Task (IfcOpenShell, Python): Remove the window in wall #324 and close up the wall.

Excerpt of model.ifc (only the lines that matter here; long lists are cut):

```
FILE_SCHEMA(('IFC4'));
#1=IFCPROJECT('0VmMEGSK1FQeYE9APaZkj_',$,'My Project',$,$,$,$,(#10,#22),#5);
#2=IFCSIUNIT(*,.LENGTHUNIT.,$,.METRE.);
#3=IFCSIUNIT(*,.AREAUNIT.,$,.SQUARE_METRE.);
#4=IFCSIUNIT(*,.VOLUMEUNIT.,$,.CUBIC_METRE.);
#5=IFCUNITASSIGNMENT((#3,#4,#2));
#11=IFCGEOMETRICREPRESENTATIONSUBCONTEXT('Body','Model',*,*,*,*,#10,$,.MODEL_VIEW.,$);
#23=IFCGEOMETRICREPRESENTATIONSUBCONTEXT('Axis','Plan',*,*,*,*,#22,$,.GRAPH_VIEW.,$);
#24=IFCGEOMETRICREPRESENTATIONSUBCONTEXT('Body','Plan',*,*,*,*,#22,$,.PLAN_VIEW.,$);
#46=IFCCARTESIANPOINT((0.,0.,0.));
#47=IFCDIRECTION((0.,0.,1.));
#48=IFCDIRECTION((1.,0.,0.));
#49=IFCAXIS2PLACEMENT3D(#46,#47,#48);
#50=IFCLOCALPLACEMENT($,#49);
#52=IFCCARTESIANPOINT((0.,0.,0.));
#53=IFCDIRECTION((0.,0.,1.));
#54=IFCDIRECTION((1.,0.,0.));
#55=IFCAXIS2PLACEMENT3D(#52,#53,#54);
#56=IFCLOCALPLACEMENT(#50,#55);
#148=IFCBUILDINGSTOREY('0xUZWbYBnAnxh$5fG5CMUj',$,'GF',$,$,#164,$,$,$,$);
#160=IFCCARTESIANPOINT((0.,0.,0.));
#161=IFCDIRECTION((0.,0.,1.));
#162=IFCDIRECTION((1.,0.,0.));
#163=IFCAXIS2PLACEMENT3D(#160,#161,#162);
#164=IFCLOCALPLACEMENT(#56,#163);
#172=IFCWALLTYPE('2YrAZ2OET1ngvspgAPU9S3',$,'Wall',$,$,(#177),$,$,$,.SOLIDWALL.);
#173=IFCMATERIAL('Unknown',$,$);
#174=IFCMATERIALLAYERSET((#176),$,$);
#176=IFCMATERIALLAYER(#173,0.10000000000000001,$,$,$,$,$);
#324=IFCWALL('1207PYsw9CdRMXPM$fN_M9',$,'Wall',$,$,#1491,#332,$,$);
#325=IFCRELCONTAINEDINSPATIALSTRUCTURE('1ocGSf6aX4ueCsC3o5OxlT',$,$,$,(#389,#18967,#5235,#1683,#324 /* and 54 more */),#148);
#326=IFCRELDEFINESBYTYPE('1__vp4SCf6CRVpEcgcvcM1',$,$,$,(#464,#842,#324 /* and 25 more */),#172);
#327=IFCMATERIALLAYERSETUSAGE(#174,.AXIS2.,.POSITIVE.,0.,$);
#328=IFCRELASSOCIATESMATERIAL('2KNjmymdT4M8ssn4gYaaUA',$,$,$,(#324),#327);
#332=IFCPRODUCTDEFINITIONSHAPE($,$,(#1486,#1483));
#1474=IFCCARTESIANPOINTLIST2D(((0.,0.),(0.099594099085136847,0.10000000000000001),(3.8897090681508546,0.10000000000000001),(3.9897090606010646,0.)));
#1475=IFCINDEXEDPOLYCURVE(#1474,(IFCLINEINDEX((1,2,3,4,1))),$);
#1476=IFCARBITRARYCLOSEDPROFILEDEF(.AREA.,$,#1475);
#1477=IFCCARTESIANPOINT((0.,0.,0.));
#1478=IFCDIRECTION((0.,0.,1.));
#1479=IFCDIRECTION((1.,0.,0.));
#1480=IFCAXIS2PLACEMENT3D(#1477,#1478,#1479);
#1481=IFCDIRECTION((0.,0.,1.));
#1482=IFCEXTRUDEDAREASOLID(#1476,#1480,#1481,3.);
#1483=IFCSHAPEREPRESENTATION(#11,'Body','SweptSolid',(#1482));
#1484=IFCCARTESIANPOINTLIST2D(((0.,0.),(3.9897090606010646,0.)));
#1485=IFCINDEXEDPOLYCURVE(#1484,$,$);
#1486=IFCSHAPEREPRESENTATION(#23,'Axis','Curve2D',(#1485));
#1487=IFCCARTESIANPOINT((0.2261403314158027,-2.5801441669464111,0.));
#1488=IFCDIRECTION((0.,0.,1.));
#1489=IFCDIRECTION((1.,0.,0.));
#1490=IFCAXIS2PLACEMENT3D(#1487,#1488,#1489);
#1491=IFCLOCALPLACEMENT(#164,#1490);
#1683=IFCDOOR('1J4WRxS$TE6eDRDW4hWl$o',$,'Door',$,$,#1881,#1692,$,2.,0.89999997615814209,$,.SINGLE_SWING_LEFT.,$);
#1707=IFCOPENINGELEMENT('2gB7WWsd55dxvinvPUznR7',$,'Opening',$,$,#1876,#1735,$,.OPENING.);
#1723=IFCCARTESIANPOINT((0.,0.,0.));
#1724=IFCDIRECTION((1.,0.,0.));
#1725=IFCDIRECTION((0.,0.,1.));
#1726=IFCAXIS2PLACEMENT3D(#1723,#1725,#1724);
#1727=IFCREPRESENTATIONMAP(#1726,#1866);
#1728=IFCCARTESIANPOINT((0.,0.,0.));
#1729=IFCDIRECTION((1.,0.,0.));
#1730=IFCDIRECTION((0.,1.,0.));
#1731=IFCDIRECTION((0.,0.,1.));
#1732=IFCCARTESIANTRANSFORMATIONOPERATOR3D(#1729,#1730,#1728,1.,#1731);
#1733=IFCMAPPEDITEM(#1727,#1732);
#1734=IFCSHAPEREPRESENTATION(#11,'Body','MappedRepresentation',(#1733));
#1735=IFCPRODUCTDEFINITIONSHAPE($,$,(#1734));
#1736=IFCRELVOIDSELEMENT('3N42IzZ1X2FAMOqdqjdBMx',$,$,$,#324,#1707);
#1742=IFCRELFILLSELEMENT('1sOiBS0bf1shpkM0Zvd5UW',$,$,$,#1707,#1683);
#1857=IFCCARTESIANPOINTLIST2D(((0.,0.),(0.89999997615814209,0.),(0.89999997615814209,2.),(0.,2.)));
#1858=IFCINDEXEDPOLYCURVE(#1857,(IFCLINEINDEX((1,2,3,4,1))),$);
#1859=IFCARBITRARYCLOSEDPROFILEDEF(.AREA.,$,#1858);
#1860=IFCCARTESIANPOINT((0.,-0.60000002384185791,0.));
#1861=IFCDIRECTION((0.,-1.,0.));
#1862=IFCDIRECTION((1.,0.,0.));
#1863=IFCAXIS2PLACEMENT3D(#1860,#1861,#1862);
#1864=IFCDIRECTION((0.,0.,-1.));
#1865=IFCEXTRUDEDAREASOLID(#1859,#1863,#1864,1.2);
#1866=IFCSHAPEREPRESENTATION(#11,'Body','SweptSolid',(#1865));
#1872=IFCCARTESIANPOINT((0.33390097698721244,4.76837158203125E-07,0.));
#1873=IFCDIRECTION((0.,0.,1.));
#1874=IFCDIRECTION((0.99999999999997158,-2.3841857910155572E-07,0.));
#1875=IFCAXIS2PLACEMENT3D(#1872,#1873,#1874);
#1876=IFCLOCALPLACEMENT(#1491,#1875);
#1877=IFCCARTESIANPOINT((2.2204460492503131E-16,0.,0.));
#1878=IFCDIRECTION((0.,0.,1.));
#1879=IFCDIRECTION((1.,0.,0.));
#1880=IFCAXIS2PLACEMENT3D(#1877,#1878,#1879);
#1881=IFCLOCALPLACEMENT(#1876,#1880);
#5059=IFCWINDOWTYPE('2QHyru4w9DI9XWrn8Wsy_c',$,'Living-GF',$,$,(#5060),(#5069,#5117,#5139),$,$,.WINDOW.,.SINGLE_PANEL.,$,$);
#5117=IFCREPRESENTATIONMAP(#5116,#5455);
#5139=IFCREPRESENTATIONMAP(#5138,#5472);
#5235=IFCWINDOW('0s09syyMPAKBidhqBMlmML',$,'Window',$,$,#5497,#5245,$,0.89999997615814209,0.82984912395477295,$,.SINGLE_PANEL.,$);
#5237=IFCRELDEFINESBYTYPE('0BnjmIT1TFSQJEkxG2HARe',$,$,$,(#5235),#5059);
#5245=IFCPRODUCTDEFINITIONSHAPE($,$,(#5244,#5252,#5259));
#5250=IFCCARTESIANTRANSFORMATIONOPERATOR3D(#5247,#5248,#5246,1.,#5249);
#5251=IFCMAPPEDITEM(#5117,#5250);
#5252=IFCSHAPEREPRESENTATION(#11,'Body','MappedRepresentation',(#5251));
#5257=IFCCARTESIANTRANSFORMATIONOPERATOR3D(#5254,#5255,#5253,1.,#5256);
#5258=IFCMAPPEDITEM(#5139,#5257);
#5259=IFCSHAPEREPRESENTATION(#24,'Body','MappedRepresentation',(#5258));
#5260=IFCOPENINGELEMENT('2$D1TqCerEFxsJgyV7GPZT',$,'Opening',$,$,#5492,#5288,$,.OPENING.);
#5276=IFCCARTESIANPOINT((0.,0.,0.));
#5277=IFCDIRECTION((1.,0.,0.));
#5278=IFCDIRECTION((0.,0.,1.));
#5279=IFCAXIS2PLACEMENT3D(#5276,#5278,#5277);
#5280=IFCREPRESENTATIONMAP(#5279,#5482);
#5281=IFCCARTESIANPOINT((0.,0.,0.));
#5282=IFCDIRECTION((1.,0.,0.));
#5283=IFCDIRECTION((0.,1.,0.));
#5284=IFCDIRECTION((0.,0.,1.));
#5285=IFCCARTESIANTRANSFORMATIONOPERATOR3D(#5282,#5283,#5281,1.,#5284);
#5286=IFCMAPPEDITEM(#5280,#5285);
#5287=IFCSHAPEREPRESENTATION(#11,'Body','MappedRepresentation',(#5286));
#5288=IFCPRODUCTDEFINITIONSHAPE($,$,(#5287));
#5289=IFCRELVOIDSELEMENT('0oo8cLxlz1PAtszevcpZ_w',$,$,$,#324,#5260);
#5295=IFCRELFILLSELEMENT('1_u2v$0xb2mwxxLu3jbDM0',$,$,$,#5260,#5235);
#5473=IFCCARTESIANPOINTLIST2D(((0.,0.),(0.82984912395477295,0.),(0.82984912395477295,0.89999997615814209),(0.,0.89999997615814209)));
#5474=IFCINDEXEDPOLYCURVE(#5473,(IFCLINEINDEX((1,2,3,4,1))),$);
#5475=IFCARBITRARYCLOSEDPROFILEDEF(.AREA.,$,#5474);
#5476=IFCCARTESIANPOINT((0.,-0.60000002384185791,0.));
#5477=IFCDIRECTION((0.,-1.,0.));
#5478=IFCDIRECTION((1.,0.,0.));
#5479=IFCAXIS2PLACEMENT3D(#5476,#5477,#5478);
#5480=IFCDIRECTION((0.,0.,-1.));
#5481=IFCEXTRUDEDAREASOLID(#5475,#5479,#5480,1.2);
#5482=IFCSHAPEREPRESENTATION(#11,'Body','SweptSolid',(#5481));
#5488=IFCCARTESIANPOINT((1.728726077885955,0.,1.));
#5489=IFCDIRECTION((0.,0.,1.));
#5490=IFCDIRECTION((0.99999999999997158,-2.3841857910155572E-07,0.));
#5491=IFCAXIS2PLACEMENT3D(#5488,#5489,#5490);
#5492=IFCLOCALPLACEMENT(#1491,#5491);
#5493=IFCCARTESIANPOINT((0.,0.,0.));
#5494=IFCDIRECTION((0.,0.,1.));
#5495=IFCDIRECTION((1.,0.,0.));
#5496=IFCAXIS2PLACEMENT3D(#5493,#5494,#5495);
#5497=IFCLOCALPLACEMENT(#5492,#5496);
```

```python
import ifcopenshell
import ifcopenshell.api.feature
import ifcopenshell.api.root
import ifcopenshell.geom
import ifcopenshell.util.shape

model = ifcopenshell.open("model.ifc")
settings = ifcopenshell.geom.settings()


def volume(element):
    """Net volume in cubic metres, openings subtracted."""
    shape = ifcopenshell.geom.create_shape(settings, element)
    return ifcopenshell.util.shape.get_volume(shape.geometry)


window = model.by_id(5235)
opening = window.FillsVoids[0].RelatingOpeningElement
wall = opening.VoidsElements[0].RelatingBuildingElement
before = volume(wall)

ifcopenshell.api.root.remove_product(model, product=window)
ifcopenshell.api.feature.remove_feature(model, feature=opening)

after = volume(wall)

print(f"wall volume {before:.3f} -> {after:.3f} m3")

model.write("model-out.ifc")
```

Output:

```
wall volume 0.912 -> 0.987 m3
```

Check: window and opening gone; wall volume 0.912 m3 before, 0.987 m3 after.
